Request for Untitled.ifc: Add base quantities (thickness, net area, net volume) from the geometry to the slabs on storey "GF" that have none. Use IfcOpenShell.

First a look at what the model holds.

```python
import ifcopenshell
import ifcopenshell.util.element
import ifcopenshell.util.unit

model = ifcopenshell.open("Untitled.ifc")
print(model.schema)
for unit_type in ("LENGTHUNIT", "AREAUNIT", "VOLUMEUNIT"):
    print(unit_type, ifcopenshell.util.unit.calculate_unit_scale(model, unit_type))
storey = next(s for s in model.by_type("IfcBuildingStorey") if s.Name == "GF")
slabs = [e for e in ifcopenshell.util.element.get_decomposition(storey) if e.is_a("IfcSlab")]
for e in sorted(slabs, key=lambda e: e.id()):
    print(e.id(), e.is_a(), e.Name, list(ifcopenshell.util.element.get_psets(e, qtos_only=True)), sep=" | ")
```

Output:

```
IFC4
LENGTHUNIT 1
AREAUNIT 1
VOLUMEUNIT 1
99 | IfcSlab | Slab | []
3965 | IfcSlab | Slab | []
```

```python
import ifcopenshell
import ifcopenshell.api.pset
import ifcopenshell.geom
import ifcopenshell.util.element
import ifcopenshell.util.shape
import ifcopenshell.util.unit

model = ifcopenshell.open("Untitled.ifc")
unit_scale = ifcopenshell.util.unit.calculate_unit_scale(model)
area_scale = ifcopenshell.util.unit.calculate_unit_scale(model, "AREAUNIT")
volume_scale = ifcopenshell.util.unit.calculate_unit_scale(model, "VOLUMEUNIT")
settings = ifcopenshell.geom.settings()

storey = next(s for s in model.by_type("IfcBuildingStorey") if s.Name == "GF")
slabs = [e for e in ifcopenshell.util.element.get_decomposition(storey) if e.is_a("IfcSlab")]

for e in sorted(slabs, key=lambda e: e.id()):
    if ifcopenshell.util.element.get_psets(e, qtos_only=True, should_inherit=False):
        continue
    # Geometry comes back in metres, in the element's own axes.
    shape = ifcopenshell.geom.create_shape(settings, e)
    values = {
        "Width": ifcopenshell.util.shape.get_z(shape.geometry) / unit_scale,
        "NetArea": ifcopenshell.util.shape.get_footprint_area(shape.geometry) / area_scale,
        "NetVolume": ifcopenshell.util.shape.get_volume(shape.geometry) / volume_scale,
    }
    qto = ifcopenshell.api.pset.add_qto(model, product=e, name="Qto_SlabBaseQuantities")
    ifcopenshell.api.pset.edit_qto(model, qto=qto, properties=values)
    print(e.id(), {k: round(v, 3) for k, v in values.items()})

model.write("Untitled-out.ifc")
```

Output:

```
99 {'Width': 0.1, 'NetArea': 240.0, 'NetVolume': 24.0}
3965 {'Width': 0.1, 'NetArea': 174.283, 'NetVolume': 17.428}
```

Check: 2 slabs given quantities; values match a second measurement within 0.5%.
